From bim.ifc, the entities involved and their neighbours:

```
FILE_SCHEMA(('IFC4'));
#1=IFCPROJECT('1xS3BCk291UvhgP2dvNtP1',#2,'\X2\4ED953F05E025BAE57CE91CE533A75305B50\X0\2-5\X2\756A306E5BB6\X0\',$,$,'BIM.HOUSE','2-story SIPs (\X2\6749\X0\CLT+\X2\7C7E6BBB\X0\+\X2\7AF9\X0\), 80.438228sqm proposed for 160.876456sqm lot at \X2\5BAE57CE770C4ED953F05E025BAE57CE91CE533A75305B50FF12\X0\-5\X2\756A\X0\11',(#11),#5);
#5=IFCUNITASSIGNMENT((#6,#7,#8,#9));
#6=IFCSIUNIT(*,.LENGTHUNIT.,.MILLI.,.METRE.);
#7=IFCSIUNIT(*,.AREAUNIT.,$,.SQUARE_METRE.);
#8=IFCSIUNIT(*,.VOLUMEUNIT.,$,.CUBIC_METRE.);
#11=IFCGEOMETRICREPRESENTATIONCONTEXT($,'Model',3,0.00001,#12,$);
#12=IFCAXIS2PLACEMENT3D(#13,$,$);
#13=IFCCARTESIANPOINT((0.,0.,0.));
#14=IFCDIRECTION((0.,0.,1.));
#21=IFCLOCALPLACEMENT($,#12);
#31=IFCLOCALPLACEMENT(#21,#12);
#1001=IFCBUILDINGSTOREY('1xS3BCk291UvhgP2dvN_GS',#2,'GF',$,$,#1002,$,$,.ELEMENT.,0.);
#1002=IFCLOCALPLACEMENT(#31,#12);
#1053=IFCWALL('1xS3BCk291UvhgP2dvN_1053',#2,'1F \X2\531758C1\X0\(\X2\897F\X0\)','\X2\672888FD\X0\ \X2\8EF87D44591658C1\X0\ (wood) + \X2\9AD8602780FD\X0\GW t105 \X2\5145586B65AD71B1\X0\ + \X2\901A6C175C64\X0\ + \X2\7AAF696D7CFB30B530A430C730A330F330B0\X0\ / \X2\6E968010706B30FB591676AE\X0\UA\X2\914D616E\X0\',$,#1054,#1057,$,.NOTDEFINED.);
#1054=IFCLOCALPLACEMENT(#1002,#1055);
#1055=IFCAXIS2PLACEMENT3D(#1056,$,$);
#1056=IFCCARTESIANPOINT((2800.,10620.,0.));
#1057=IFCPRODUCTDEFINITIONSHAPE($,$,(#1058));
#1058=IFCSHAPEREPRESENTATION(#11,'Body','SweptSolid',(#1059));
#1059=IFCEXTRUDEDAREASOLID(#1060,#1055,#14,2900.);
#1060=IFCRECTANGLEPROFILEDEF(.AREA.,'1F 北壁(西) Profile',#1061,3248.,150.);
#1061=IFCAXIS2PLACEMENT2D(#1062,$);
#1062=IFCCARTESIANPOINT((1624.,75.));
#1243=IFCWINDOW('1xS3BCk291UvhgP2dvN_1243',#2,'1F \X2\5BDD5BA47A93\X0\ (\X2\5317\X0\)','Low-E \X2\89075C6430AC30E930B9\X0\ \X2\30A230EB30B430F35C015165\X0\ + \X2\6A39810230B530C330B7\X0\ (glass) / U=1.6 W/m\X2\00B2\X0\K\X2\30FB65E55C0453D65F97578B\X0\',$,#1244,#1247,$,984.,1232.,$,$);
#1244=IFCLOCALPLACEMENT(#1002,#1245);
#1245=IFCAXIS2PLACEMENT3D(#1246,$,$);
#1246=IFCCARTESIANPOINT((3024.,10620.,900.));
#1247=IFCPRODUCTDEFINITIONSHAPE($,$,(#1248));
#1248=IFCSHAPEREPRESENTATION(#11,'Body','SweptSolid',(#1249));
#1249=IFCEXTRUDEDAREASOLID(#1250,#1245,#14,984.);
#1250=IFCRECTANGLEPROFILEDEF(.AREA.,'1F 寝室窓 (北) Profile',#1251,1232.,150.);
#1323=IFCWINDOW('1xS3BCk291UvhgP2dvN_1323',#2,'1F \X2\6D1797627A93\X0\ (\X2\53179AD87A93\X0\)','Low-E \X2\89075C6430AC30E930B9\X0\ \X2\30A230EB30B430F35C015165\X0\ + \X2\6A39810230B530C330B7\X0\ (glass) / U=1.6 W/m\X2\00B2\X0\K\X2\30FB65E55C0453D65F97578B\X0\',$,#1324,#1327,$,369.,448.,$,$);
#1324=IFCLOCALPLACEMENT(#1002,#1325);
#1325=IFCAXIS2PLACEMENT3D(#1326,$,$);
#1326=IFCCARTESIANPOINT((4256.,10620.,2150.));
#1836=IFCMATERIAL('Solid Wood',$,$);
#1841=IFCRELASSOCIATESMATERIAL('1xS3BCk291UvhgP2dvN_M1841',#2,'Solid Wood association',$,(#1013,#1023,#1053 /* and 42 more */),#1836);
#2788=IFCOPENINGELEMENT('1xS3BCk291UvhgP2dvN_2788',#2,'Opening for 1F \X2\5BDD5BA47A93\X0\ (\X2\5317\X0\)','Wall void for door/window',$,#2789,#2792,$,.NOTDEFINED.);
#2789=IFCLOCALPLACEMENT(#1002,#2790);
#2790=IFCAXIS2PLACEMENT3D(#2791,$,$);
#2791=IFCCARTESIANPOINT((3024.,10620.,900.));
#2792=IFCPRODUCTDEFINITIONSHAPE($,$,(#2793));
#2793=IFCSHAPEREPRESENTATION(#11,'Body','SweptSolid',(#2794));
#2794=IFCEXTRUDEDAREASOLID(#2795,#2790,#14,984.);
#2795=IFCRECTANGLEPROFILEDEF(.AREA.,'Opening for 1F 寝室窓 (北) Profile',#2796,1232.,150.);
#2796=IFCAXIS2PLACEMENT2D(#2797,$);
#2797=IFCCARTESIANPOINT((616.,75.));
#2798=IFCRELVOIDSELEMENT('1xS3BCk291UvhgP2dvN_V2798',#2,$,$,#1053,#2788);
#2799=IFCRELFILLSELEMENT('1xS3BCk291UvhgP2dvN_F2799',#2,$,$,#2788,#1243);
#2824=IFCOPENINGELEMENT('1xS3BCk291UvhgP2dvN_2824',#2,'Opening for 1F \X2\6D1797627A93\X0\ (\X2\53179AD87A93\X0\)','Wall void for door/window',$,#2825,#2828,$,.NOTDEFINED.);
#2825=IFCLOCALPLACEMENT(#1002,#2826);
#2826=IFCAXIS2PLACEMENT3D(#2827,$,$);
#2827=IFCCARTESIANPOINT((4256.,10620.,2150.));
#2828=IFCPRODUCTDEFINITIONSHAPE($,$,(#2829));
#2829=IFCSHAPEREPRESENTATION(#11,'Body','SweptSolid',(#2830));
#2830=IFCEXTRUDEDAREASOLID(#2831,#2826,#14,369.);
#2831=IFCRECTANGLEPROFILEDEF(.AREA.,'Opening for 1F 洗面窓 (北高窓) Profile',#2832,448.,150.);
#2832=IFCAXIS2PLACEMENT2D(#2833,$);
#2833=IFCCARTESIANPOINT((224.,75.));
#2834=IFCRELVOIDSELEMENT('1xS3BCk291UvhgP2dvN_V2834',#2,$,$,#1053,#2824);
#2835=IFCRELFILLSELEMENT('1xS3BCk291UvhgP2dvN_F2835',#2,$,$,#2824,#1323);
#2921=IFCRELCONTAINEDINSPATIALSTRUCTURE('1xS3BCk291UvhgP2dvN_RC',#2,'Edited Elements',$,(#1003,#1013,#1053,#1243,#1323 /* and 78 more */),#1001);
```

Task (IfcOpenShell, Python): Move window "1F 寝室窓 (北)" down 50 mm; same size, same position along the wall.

```python
import numpy as np
import ifcopenshell
import ifcopenshell.api.geometry
import ifcopenshell.util.placement
import ifcopenshell.util.unit

model = ifcopenshell.open("bim.ifc")
unit_scale = ifcopenshell.util.unit.calculate_unit_scale(model)

window = model.by_guid("1xS3BCk291UvhgP2dvN_1243")
opening = window.FillsVoids[0].RelatingOpeningElement
dz = -50.0

shift = np.array([0.0, 0.0, dz])
# The window is not placed relative to its opening, so move both.
for product in (opening, window):
    matrix = ifcopenshell.util.placement.get_local_placement(product.ObjectPlacement)
    matrix[:3, 3] += shift
    ifcopenshell.api.geometry.edit_object_placement(model, product=product, matrix=matrix, is_si=False)

print(f"moved by {dz * unit_scale:+.3f} m")

model.write("bim_rev.ifc")
```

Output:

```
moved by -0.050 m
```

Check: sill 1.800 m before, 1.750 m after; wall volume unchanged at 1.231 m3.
